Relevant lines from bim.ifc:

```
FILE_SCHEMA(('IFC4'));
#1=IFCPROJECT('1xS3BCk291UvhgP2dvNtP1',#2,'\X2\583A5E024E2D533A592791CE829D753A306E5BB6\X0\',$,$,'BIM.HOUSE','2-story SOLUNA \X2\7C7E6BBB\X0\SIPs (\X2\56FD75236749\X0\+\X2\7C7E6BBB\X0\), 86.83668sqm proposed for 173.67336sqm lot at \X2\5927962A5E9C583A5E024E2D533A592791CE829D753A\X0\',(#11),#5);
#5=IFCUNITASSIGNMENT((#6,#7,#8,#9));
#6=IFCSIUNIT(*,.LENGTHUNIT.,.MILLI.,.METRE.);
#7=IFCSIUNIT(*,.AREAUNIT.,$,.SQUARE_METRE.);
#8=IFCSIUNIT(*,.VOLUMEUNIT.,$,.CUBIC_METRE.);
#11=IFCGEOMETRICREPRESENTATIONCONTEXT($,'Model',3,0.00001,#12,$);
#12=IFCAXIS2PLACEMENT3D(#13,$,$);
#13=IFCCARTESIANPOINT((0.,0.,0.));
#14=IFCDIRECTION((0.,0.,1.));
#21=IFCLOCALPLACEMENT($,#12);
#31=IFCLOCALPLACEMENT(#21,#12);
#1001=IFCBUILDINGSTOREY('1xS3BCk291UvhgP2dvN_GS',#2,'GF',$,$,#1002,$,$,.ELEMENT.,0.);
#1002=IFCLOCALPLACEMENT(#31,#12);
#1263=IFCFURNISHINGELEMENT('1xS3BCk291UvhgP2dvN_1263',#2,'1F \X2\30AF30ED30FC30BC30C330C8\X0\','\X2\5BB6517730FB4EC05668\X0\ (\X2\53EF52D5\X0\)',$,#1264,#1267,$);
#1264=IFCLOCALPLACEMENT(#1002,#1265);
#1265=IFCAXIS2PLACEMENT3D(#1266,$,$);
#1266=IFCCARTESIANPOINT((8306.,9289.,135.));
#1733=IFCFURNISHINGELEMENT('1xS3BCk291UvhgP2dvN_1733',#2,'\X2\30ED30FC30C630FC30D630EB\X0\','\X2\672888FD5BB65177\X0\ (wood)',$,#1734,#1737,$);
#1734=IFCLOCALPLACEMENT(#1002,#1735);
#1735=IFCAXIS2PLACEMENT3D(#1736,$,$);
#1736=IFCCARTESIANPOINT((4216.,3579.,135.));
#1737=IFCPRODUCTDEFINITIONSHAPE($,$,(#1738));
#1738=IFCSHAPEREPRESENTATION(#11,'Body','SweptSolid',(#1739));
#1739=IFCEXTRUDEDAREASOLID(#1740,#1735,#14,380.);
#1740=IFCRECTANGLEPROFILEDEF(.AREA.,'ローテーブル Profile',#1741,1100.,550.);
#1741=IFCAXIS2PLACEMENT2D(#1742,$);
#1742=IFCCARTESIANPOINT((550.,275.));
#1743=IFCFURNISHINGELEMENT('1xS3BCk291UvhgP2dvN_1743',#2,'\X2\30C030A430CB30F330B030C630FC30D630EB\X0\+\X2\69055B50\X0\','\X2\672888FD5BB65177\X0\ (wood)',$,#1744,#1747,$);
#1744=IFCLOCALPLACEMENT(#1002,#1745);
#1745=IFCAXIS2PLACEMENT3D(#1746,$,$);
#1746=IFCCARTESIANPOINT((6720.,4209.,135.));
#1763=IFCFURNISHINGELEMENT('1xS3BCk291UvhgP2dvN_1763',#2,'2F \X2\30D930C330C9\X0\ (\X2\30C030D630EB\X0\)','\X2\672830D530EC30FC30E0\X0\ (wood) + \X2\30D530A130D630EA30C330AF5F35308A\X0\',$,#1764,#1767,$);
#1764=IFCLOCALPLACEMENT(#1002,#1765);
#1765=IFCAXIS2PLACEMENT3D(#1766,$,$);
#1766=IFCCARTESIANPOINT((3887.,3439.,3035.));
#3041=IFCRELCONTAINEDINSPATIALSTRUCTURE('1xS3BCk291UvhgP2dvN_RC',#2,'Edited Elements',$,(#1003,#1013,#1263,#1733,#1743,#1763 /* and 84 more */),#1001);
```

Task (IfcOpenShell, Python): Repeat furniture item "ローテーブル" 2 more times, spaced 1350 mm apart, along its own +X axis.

```python
import ifcopenshell
import ifcopenshell.api.geometry
import ifcopenshell.api.root
import ifcopenshell.util.element
import ifcopenshell.util.placement
import ifcopenshell.util.unit

model = ifcopenshell.open("bim.ifc")
unit_scale = ifcopenshell.util.unit.calculate_unit_scale(model)


def reuse_history(source, copy):
    """copy_class also copies each property set's owner history, people and application; keep the originals."""
    for rel in copy.IsDefinedBy:
        if rel.is_a("IfcRelDefinesByProperties") and (history := rel.RelatingPropertyDefinition.OwnerHistory):
            rel.RelatingPropertyDefinition.OwnerHistory = source.OwnerHistory
            ifcopenshell.util.element.remove_deep2(model, history)


source = model.by_id(1733)
base = ifcopenshell.util.placement.get_local_placement(source.ObjectPlacement)
step = base[:3, 0] * 1.35 / unit_scale

for i in range(1, 3):
    copy = ifcopenshell.api.root.copy_class(model, product=source)
    copy.Representation = ifcopenshell.util.element.copy_deep(
        model, source.Representation, exclude=["IfcGeometricRepresentationContext", "IfcRepresentationMap"]
    )
    reuse_history(source, copy)
    matrix = base.copy()
    matrix[:3, 3] += i * step
    print("added at", matrix[:3, 3].round(3) + 0.0)
    ifcopenshell.api.geometry.edit_object_placement(model, product=copy, matrix=matrix, is_si=False)

model.write("bim_updated.ifc")
```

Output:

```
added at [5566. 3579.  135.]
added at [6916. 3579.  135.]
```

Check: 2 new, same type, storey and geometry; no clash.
